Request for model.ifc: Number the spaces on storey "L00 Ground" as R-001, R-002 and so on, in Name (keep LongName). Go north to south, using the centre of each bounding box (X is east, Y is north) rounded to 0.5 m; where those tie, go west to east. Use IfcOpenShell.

First a look at what the model holds.

```python
import ifcopenshell
import ifcopenshell.util.element
import ifcopenshell.util.placement

model = ifcopenshell.open("model.ifc")
print(model.schema)
storey = next(s for s in model.by_type("IfcBuildingStorey") if s.Name == "L00 Ground")
spaces = [e for e in ifcopenshell.util.element.get_decomposition(storey) if e.is_a("IfcSpace")]
for e in sorted(spaces, key=lambda e: e.id()):
    origin = ifcopenshell.util.placement.get_local_placement(e.ObjectPlacement)[:3, 3]
    print(e.id(), e.Name, e.LongName, origin.round(2) + 0.0, sep=" | ")
```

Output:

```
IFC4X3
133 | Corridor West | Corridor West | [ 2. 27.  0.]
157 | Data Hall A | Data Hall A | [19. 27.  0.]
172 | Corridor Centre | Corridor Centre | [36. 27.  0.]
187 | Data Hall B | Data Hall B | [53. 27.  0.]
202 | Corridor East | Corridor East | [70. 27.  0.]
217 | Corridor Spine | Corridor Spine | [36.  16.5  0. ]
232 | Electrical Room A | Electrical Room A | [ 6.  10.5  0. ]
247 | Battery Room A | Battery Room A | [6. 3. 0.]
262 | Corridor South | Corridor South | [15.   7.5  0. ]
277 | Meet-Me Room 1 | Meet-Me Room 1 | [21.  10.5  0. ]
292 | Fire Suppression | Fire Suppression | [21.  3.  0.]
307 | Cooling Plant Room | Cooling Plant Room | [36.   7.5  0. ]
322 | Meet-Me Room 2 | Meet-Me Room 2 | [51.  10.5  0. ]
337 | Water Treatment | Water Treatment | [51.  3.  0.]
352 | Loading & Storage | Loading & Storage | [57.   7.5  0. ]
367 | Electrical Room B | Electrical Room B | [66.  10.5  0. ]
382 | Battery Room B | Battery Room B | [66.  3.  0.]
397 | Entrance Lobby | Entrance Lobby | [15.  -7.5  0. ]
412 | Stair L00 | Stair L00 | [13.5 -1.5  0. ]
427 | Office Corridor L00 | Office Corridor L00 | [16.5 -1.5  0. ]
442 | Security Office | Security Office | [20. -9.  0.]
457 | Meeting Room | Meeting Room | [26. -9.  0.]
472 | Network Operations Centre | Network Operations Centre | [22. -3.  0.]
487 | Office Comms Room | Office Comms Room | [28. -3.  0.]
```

```python
import ifcopenshell
import ifcopenshell.geom
import ifcopenshell.util.element
import ifcopenshell.util.shape

model = ifcopenshell.open("model.ifc")
settings = ifcopenshell.geom.settings()
settings.set("use-world-coords", True)


def centre(element):
    shape = ifcopenshell.geom.create_shape(settings, element)
    return ifcopenshell.util.shape.get_bbox_centroid(shape.geometry)


storey = next(s for s in model.by_type("IfcBuildingStorey") if s.Name == "L00 Ground")
spaces = [e for e in ifcopenshell.util.element.get_decomposition(storey) if e.is_a("IfcSpace")]

# Insertion points can sit at a corner or the storey origin, so sort by the geometry (in metres).
centres = {e: centre(e) for e in spaces}
spaces.sort(key=lambda e: (-round(centres[e][1] / 0.5), centres[e][0]))

for i, e in enumerate(spaces, start=1):
    number = f"R-0{i:02d}"
    e.Name = number
    print(e.id(), number)

model.write("model_rev.ifc")
```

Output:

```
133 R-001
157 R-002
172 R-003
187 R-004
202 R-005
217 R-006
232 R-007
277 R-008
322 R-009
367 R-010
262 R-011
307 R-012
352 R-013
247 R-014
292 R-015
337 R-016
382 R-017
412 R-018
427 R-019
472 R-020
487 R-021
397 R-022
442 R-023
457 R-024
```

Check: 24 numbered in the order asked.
